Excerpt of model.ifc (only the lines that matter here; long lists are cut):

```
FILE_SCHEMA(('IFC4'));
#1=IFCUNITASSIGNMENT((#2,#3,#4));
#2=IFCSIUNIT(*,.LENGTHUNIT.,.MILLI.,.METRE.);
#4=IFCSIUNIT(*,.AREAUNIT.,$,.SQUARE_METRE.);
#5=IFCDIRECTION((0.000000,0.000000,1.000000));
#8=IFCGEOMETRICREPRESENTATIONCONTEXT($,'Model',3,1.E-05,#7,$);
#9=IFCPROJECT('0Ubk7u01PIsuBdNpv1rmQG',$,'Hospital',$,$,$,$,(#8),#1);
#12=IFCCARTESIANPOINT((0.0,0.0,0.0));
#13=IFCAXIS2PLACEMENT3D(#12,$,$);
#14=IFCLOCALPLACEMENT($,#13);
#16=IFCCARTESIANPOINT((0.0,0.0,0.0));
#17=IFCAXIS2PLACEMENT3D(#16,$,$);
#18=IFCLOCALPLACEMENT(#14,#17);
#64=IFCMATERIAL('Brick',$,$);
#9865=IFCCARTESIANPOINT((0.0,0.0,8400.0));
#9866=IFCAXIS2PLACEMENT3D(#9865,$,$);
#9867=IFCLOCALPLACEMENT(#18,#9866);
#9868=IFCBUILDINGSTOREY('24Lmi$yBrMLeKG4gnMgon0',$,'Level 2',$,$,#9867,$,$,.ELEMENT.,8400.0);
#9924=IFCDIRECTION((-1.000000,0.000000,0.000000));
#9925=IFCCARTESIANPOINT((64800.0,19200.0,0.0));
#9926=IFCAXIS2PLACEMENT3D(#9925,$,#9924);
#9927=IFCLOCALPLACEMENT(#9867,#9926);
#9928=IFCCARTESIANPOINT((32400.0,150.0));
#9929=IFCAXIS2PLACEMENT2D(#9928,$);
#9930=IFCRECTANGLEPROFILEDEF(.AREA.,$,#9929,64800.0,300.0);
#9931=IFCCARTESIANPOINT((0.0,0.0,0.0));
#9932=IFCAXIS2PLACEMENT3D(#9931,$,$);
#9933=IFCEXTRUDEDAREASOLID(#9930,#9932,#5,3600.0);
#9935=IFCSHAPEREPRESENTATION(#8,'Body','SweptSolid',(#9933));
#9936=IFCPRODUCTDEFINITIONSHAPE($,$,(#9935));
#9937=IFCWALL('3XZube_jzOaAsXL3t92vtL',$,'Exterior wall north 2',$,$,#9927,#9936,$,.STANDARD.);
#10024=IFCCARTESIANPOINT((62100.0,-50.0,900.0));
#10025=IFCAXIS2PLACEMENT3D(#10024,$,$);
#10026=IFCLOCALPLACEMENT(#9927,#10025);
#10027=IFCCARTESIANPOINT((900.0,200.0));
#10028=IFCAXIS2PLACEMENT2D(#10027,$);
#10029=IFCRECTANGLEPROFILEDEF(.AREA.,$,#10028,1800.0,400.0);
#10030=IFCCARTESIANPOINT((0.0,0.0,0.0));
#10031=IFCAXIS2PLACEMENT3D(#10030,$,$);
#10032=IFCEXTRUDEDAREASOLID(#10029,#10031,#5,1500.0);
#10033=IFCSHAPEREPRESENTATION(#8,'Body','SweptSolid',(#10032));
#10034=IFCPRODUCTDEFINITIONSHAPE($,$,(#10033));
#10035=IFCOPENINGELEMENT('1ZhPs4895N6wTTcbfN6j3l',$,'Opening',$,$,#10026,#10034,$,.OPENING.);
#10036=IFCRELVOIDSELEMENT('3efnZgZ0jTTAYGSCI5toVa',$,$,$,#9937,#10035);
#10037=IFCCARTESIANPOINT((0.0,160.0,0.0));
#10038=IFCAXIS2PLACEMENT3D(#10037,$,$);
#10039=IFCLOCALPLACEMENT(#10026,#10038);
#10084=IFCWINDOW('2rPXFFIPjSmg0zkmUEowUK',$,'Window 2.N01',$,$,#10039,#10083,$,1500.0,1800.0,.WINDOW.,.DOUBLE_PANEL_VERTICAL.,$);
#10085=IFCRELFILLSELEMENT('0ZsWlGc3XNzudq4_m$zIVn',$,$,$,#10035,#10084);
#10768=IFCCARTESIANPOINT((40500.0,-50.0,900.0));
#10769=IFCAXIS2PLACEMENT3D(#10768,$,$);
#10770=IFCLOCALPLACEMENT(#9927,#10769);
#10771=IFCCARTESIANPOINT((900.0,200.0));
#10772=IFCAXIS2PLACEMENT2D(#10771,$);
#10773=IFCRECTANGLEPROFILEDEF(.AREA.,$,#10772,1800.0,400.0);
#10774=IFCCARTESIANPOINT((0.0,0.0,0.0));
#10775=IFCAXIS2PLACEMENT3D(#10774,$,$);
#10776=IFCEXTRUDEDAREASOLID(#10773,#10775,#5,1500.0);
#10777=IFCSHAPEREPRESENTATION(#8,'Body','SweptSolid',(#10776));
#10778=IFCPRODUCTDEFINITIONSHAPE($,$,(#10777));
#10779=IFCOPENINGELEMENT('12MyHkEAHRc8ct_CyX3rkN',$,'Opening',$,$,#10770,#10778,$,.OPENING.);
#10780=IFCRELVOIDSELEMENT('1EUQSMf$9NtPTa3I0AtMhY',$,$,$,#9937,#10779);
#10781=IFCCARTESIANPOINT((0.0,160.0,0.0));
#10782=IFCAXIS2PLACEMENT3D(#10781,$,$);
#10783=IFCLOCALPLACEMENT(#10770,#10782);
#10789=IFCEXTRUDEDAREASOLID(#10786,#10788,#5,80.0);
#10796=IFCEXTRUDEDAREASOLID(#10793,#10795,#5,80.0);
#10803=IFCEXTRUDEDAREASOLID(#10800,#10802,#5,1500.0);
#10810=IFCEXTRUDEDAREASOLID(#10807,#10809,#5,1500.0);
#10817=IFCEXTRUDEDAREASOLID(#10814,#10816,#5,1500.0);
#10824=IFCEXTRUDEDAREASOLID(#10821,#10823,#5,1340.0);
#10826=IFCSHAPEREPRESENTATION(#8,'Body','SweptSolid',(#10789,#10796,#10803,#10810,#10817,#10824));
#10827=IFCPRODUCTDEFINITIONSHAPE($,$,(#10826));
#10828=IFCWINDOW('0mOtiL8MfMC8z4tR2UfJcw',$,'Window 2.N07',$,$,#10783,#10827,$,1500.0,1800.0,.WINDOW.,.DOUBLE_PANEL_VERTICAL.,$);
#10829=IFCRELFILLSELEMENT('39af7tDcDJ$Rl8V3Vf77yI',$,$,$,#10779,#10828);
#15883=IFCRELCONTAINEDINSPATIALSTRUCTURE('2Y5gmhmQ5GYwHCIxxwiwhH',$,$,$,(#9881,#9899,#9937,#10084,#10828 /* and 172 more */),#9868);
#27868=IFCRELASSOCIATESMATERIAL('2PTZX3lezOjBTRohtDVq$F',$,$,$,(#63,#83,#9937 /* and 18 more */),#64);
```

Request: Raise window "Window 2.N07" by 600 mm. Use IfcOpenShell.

```python
import numpy as np
import ifcopenshell
import ifcopenshell.api.geometry
import ifcopenshell.util.placement
import ifcopenshell.util.unit

model = ifcopenshell.open("model.ifc")
unit_scale = ifcopenshell.util.unit.calculate_unit_scale(model)

window = model.by_guid("0mOtiL8MfMC8z4tR2UfJcw")
opening = window.FillsVoids[0].RelatingOpeningElement
dz = 0.6 / unit_scale

shift = np.array([0.0, 0.0, dz])
# The window is placed relative to its opening, so it follows when the opening moves.
matrix = ifcopenshell.util.placement.get_local_placement(opening.ObjectPlacement)
matrix[:3, 3] += shift
ifcopenshell.api.geometry.edit_object_placement(
    model, product=opening, matrix=matrix, is_si=False, should_transform_children=True
)

print(f"moved by {dz * unit_scale:+.3f} m")

model.write("model_edited.ifc")
```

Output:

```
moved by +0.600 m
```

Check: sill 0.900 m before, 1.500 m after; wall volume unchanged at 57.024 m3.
